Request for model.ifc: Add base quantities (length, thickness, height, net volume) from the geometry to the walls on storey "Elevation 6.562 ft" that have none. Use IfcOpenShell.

First a look at what the model holds.

```python
import ifcopenshell
import ifcopenshell.util.element
import ifcopenshell.util.unit

model = ifcopenshell.open("model.ifc")
print(model.schema)
for unit_type in ("LENGTHUNIT", "AREAUNIT", "VOLUMEUNIT"):
    print(unit_type, ifcopenshell.util.unit.calculate_unit_scale(model, unit_type))
storey = next(s for s in model.by_type("IfcBuildingStorey") if s.Name == "Elevation 6.562 ft")
walls = [e for e in ifcopenshell.util.element.get_decomposition(storey) if e.is_a("IfcWall")]
for e in sorted(walls, key=lambda e: e.id()):
    print(e.id(), e.is_a(), e.Name, list(ifcopenshell.util.element.get_psets(e, qtos_only=True)), sep=" | ")
```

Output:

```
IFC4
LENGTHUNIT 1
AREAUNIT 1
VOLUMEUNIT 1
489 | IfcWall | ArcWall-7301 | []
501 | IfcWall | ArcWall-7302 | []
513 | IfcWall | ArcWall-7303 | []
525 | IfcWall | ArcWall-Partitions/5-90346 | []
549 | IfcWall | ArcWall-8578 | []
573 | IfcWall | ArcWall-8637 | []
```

```python
import ifcopenshell
import ifcopenshell.api.pset
import ifcopenshell.geom
import ifcopenshell.util.element
import ifcopenshell.util.shape
import ifcopenshell.util.unit

model = ifcopenshell.open("model.ifc")
unit_scale = ifcopenshell.util.unit.calculate_unit_scale(model)
volume_scale = ifcopenshell.util.unit.calculate_unit_scale(model, "VOLUMEUNIT")
settings = ifcopenshell.geom.settings()

storey = next(s for s in model.by_type("IfcBuildingStorey") if s.Name == "Elevation 6.562 ft")
walls = [e for e in ifcopenshell.util.element.get_decomposition(storey) if e.is_a("IfcWall")]

for e in sorted(walls, key=lambda e: e.id()):
    if ifcopenshell.util.element.get_psets(e, qtos_only=True, should_inherit=False):
        continue
    # Geometry comes back in metres, in the element's own axes.
    shape = ifcopenshell.geom.create_shape(settings, e)
    values = {
        "Length": ifcopenshell.util.shape.get_x(shape.geometry) / unit_scale,
        "Width": ifcopenshell.util.shape.get_y(shape.geometry) / unit_scale,
        "Height": ifcopenshell.util.shape.get_z(shape.geometry) / unit_scale,
        "NetVolume": ifcopenshell.util.shape.get_volume(shape.geometry) / volume_scale,
    }
    qto = ifcopenshell.api.pset.add_qto(model, product=e, name="Qto_WallBaseQuantities")
    ifcopenshell.api.pset.edit_qto(model, qto=qto, properties=values)
    print(e.id(), {k: round(v, 3) for k, v in values.items()})

model.write("model_v2.ifc")
```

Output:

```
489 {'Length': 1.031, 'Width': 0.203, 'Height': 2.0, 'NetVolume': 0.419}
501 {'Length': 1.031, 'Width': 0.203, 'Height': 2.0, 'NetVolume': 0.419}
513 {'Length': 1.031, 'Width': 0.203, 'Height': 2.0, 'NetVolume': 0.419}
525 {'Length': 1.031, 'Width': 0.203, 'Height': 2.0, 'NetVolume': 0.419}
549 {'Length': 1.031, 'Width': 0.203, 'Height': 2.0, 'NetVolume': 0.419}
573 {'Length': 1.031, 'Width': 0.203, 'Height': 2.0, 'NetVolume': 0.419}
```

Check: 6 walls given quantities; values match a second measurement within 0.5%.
